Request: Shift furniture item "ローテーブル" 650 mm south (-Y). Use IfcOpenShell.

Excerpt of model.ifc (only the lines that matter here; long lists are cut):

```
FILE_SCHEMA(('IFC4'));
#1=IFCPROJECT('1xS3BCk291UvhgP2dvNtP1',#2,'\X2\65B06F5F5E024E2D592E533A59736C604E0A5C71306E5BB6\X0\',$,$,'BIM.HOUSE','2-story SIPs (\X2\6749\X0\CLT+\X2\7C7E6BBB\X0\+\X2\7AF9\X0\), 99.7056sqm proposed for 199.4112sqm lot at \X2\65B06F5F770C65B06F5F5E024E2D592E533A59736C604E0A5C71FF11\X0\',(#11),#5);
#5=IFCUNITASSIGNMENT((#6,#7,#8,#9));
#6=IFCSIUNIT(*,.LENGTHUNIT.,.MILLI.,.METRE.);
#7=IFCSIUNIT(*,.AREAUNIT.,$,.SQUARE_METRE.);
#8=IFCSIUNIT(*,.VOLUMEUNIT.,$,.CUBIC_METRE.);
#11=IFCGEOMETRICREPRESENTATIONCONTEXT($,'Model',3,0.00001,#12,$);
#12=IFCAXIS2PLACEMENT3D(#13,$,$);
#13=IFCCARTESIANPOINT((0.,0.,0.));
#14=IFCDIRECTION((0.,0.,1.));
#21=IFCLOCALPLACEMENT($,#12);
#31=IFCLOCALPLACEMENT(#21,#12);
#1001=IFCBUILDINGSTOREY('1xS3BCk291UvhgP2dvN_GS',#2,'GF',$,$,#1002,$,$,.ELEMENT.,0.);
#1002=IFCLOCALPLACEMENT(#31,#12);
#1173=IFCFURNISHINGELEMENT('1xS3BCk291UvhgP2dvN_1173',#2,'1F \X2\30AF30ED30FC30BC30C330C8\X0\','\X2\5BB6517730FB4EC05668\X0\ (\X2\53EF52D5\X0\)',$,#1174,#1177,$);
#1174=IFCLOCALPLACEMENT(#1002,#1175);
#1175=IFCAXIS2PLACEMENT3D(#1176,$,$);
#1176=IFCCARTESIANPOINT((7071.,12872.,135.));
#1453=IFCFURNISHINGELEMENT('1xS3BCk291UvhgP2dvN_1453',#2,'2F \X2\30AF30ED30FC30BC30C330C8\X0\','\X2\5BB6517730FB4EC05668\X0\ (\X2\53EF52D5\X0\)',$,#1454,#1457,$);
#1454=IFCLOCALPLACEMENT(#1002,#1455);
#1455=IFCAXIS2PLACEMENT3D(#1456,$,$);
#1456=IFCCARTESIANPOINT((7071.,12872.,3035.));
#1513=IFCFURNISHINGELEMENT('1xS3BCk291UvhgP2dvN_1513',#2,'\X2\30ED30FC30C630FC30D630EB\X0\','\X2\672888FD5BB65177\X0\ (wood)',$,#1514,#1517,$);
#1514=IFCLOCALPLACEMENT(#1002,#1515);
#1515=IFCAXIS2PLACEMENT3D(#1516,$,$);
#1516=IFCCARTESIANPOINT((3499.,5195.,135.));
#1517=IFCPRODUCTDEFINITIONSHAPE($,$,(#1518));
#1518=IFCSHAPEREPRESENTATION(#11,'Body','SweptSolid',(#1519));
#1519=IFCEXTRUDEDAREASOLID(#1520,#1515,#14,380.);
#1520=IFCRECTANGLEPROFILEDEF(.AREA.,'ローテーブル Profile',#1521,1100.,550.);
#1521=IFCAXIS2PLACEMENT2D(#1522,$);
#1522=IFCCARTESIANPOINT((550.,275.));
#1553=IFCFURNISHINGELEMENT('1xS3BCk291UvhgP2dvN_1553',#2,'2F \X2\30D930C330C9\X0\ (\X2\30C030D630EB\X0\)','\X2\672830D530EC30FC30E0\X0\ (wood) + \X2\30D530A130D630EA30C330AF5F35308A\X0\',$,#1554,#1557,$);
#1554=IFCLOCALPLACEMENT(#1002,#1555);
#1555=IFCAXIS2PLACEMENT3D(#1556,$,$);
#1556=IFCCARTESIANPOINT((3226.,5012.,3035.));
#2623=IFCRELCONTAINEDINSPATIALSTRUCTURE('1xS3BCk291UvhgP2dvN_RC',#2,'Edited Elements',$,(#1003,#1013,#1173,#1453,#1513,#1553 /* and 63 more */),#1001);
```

```python
import ifcopenshell
import ifcopenshell.api.geometry
import ifcopenshell.util.placement
import ifcopenshell.util.unit

model = ifcopenshell.open("model.ifc")
unit_scale = ifcopenshell.util.unit.calculate_unit_scale(model)

item = model.by_id(1513)
matrix = ifcopenshell.util.placement.get_local_placement(item.ObjectPlacement)
matrix[1, 3] -= 0.65 / unit_scale
ifcopenshell.api.geometry.edit_object_placement(model, product=item, matrix=matrix, is_si=False)

print(ifcopenshell.util.placement.get_local_placement(item.ObjectPlacement).round(3) + 0.0)

model.write("model-out.ifc")
```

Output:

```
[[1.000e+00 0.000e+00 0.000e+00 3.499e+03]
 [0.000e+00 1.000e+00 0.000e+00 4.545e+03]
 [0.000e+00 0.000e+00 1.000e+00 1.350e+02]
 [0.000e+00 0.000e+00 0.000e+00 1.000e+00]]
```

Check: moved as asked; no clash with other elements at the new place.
